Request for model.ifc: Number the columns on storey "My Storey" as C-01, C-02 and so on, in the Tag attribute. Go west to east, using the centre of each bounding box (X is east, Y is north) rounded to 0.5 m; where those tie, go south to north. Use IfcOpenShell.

First a look at what the model holds.

```python
import ifcopenshell
import ifcopenshell.util.element
import ifcopenshell.util.placement

model = ifcopenshell.open("model.ifc")
print(model.schema)
storey = next(s for s in model.by_type("IfcBuildingStorey") if s.Name == "My Storey")
columns = [e for e in ifcopenshell.util.element.get_decomposition(storey) if e.is_a("IfcColumn")]
for e in sorted(columns, key=lambda e: e.id()):
    origin = ifcopenshell.util.placement.get_local_placement(e.ObjectPlacement)[:3, 3]
    print(e.id(), e.Tag, e.Name, origin.round(2) + 0.0, sep=" | ")
```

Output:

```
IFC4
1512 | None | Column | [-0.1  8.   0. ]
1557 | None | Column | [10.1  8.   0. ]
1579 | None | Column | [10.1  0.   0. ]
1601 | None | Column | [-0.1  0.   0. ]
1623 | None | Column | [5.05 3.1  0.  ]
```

```python
import ifcopenshell
import ifcopenshell.geom
import ifcopenshell.util.element
import ifcopenshell.util.shape

model = ifcopenshell.open("model.ifc")
settings = ifcopenshell.geom.settings()
settings.set("use-world-coords", True)


def centre(element):
    shape = ifcopenshell.geom.create_shape(settings, element)
    return ifcopenshell.util.shape.get_bbox_centroid(shape.geometry)


storey = next(s for s in model.by_type("IfcBuildingStorey") if s.Name == "My Storey")
columns = [e for e in ifcopenshell.util.element.get_decomposition(storey) if e.is_a("IfcColumn")]

# Insertion points can sit at a corner or the storey origin, so sort by the geometry (in metres).
centres = {e: centre(e) for e in columns}
columns.sort(key=lambda e: (round(centres[e][0] / 0.5), centres[e][1]))

for i, e in enumerate(columns, start=1):
    number = f"C-{i:02d}"
    e.Tag = number
    print(e.id(), number)

model.write("model_v2.ifc")
```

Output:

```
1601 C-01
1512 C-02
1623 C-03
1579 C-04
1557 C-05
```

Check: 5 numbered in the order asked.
